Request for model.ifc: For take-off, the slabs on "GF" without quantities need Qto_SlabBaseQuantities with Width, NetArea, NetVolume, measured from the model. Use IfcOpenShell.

First a look at what the model holds.

```python
import ifcopenshell
import ifcopenshell.util.element
import ifcopenshell.util.unit

model = ifcopenshell.open("model.ifc")
print(model.schema)
for unit_type in ("LENGTHUNIT", "AREAUNIT", "VOLUMEUNIT"):
    print(unit_type, ifcopenshell.util.unit.calculate_unit_scale(model, unit_type))
storey = next(s for s in model.by_type("IfcBuildingStorey") if s.Name == "GF")
slabs = [e for e in ifcopenshell.util.element.get_decomposition(storey) if e.is_a("IfcSlab")]
for e in sorted(slabs, key=lambda e: e.id()):
    print(e.id(), e.is_a(), e.Name, list(ifcopenshell.util.element.get_psets(e, qtos_only=True)), sep=" | ")
```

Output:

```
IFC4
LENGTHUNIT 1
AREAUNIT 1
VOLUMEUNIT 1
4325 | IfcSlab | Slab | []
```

```python
import ifcopenshell
import ifcopenshell.api.pset
import ifcopenshell.geom
import ifcopenshell.util.element
import ifcopenshell.util.shape
import ifcopenshell.util.unit

model = ifcopenshell.open("model.ifc")
unit_scale = ifcopenshell.util.unit.calculate_unit_scale(model)
area_scale = ifcopenshell.util.unit.calculate_unit_scale(model, "AREAUNIT")
volume_scale = ifcopenshell.util.unit.calculate_unit_scale(model, "VOLUMEUNIT")
settings = ifcopenshell.geom.settings()

storey = next(s for s in model.by_type("IfcBuildingStorey") if s.Name == "GF")
slabs = [e for e in ifcopenshell.util.element.get_decomposition(storey) if e.is_a("IfcSlab")]

for e in sorted(slabs, key=lambda e: e.id()):
    if ifcopenshell.util.element.get_psets(e, qtos_only=True, should_inherit=False):
        continue
    # Geometry comes back in metres, in the element's own axes.
    shape = ifcopenshell.geom.create_shape(settings, e)
    values = {
        "Width": ifcopenshell.util.shape.get_z(shape.geometry) / unit_scale,
        "NetArea": ifcopenshell.util.shape.get_footprint_area(shape.geometry) / area_scale,
        "NetVolume": ifcopenshell.util.shape.get_volume(shape.geometry) / volume_scale,
    }
    qto = ifcopenshell.api.pset.add_qto(model, product=e, name="Qto_SlabBaseQuantities")
    ifcopenshell.api.pset.edit_qto(model, qto=qto, properties=values)
    print(e.id(), {k: round(v, 3) for k, v in values.items()})

model.write("model_rev.ifc")
```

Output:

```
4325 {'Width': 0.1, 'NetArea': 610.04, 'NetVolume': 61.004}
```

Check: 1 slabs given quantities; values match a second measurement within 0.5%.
